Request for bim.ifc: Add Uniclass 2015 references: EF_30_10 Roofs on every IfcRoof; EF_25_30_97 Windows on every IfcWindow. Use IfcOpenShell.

First a look at what the model holds.

```python
import ifcopenshell

model = ifcopenshell.open("bim.ifc")
print(model.schema)
print("classifications:", [c.Name for c in model.by_type("IfcClassification")])
for ifc_class in ("IfcDoor", "IfcRoof", "IfcStair", "IfcWall", "IfcWindow"):
    print(ifc_class, len(model.by_type(ifc_class)))
```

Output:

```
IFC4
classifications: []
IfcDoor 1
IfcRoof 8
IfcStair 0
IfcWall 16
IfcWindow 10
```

```python
import ifcopenshell
import ifcopenshell.api.classification

model = ifcopenshell.open("bim.ifc")

system = ifcopenshell.api.classification.add_classification(model, classification="Uniclass 2015")

codes = {
    "IfcRoof": ("EF_30_10", "Roofs"),
    "IfcWindow": ("EF_25_30_97", "Windows"),
}
for ifc_class, (code, name) in codes.items():
    products = model.by_type(ifc_class)
    ifcopenshell.api.classification.add_reference(
        model, products=products, classification=system, identification=code, name=name
    )
    print(code, len(products))

model.write("bim-out.ifc")
```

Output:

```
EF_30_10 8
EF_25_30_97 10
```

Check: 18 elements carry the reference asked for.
